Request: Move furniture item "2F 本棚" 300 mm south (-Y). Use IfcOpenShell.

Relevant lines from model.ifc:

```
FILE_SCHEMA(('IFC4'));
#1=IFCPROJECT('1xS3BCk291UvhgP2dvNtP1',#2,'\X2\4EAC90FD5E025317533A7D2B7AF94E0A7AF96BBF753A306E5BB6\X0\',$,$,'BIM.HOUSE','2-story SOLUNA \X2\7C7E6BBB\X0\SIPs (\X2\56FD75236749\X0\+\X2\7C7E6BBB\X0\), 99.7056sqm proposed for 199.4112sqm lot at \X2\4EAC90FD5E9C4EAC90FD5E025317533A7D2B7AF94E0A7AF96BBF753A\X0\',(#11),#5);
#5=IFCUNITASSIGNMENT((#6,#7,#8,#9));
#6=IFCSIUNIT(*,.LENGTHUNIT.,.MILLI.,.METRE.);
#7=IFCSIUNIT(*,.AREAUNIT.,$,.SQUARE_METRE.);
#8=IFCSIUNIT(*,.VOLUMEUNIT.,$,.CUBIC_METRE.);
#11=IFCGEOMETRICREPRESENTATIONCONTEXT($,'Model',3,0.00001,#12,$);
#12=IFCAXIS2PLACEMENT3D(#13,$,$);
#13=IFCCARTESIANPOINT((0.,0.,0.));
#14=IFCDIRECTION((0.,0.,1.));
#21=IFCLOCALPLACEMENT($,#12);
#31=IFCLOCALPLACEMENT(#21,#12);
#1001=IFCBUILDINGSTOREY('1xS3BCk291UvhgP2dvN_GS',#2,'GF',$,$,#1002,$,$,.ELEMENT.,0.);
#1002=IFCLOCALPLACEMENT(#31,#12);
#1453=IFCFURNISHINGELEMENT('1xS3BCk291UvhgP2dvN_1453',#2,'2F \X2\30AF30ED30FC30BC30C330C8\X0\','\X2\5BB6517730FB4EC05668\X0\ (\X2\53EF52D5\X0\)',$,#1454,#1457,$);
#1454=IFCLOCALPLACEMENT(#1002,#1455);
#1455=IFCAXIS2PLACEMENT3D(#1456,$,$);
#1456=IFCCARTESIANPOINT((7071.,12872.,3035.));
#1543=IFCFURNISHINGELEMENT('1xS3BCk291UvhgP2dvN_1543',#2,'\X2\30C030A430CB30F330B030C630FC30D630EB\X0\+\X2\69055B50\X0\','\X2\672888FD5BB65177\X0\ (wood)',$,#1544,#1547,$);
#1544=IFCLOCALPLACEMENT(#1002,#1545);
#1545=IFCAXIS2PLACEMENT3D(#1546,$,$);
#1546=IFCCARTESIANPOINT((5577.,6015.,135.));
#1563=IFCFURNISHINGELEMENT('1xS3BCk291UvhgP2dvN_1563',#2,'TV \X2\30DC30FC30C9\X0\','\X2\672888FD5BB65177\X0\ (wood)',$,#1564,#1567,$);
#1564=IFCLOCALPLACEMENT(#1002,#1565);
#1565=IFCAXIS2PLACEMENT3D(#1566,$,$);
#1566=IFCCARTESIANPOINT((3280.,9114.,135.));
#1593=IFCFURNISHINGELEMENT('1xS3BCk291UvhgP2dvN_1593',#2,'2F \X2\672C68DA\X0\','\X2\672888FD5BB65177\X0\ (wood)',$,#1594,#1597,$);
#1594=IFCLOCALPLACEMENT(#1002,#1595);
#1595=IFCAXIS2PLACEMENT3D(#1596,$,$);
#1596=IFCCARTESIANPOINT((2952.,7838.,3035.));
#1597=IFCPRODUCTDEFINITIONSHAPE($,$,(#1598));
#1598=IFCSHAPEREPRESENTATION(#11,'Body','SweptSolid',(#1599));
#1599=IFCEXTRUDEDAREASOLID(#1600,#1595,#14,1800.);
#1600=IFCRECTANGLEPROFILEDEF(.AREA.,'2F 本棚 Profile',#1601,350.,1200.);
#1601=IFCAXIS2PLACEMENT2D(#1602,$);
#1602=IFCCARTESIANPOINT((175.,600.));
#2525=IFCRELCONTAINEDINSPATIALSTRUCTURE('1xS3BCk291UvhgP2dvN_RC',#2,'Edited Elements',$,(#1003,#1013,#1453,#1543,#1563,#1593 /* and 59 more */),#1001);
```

```python
import ifcopenshell
import ifcopenshell.api.geometry
import ifcopenshell.util.placement

model = ifcopenshell.open("model.ifc")

item = model.by_guid("1xS3BCk291UvhgP2dvN_1593")
matrix = ifcopenshell.util.placement.get_local_placement(item.ObjectPlacement)
matrix[1, 3] -= 300.0
ifcopenshell.api.geometry.edit_object_placement(model, product=item, matrix=matrix, is_si=False)

print(ifcopenshell.util.placement.get_local_placement(item.ObjectPlacement).round(3) + 0.0)

model.write("model_edited.ifc")
```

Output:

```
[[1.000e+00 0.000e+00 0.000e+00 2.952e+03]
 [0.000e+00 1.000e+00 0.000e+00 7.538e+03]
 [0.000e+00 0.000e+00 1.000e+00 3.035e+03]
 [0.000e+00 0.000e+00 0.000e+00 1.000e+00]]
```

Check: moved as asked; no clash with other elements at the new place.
